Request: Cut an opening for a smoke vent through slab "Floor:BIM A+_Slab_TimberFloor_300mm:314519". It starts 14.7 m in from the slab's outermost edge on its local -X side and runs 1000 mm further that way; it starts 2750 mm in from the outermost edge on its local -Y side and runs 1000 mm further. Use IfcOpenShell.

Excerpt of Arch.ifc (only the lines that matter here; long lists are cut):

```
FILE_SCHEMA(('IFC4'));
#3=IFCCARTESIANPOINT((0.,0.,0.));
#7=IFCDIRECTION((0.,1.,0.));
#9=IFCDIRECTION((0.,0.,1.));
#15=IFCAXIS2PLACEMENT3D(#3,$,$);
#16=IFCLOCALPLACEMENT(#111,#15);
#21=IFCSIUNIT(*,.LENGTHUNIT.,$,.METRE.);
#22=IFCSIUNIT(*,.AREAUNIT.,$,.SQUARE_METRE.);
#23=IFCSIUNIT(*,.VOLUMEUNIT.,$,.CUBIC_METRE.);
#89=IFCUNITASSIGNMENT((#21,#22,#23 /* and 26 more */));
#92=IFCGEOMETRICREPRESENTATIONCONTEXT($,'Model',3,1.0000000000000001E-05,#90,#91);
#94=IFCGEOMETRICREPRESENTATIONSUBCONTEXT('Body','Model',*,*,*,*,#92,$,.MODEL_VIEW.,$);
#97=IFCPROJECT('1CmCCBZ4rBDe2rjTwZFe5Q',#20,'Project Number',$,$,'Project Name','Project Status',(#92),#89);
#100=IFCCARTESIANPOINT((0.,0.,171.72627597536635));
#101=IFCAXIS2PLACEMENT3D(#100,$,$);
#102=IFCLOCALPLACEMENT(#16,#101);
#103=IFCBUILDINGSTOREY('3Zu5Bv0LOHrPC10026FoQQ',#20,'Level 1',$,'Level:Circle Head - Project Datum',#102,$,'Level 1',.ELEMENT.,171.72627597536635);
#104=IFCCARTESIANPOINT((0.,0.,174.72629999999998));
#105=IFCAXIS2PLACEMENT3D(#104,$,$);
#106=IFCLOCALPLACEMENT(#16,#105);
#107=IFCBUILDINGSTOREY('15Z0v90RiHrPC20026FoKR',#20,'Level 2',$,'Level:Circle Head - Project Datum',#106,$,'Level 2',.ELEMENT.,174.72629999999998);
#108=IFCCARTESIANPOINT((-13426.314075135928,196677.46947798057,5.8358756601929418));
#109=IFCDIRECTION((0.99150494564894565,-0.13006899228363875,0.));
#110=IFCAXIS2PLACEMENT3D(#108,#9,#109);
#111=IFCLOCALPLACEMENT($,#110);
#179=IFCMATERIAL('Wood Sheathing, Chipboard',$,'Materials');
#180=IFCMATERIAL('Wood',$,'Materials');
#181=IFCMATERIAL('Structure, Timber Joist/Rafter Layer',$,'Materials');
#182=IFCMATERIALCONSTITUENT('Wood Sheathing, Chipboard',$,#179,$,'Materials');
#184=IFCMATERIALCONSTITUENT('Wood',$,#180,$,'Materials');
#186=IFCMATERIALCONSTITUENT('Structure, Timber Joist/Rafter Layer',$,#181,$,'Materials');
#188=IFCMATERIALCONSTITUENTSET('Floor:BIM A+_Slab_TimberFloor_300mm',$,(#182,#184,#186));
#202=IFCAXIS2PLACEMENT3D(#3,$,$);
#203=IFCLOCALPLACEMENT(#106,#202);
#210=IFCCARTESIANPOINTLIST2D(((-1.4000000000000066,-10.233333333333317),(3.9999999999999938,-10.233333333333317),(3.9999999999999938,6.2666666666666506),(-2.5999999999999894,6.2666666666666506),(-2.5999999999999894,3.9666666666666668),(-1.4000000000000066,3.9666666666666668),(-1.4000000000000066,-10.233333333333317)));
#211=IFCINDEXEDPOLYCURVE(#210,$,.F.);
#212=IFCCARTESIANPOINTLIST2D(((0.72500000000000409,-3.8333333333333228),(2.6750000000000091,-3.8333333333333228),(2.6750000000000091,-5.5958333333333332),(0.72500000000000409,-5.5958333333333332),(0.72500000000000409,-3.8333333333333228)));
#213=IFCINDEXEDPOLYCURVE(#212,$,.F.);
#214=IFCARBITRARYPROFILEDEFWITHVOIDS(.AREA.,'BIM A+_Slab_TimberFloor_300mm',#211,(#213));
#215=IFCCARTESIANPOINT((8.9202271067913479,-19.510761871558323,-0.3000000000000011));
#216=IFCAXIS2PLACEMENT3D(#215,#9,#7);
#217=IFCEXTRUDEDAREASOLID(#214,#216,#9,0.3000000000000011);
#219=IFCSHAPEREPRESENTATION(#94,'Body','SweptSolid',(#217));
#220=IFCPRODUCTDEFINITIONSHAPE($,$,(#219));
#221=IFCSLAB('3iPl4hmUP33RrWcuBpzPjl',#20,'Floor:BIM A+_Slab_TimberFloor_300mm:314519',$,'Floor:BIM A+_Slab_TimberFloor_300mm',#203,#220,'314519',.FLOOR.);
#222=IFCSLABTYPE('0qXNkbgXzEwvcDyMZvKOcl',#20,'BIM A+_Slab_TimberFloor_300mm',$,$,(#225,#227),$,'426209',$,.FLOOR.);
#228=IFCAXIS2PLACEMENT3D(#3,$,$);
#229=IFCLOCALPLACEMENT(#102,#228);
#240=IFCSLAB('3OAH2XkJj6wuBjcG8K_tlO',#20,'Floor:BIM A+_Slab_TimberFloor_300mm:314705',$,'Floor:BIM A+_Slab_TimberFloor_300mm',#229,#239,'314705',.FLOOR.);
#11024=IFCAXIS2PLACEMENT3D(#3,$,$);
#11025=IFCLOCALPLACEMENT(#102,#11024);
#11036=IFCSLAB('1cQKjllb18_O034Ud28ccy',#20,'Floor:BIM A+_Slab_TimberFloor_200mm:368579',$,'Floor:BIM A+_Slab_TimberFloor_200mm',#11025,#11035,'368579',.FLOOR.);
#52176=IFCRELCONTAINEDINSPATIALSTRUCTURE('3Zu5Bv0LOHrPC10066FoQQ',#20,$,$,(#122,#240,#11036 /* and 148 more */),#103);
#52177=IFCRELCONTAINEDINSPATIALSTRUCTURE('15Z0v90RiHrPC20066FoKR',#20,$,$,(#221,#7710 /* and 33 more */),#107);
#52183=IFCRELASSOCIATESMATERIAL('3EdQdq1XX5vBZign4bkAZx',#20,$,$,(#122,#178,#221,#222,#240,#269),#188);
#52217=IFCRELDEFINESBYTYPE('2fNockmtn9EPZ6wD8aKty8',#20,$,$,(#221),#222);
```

```python
import numpy as np
import ifcopenshell
import ifcopenshell.api.feature
import ifcopenshell.api.geometry
import ifcopenshell.api.root
import ifcopenshell.geom
import ifcopenshell.util.placement
import ifcopenshell.util.representation
import ifcopenshell.util.shape
import ifcopenshell.util.unit

model = ifcopenshell.open("Arch.ifc")
unit_scale = ifcopenshell.util.unit.calculate_unit_scale(model)
settings = ifcopenshell.geom.settings()


def volume(element):
    """Net volume in cubic metres, openings subtracted."""
    shape = ifcopenshell.geom.create_shape(settings, element)
    return ifcopenshell.util.shape.get_volume(shape.geometry)


slab = model.by_guid("3iPl4hmUP33RrWcuBpzPjl")
before = volume(slab)

# Extent in the slab's own axes, in metres. The edges named are its -X and -Y sides.
slab_shape = ifcopenshell.geom.create_shape(settings, slab)
vertices = ifcopenshell.util.shape.get_vertices(slab_shape.geometry)
x_min, y_min, bottom = vertices.min(axis=0)
top = vertices[:, 2].max()

opening = ifcopenshell.api.root.create_entity(model, ifc_class="IfcOpeningElement", name="Smoke vent opening", predefined_type="OPENING")
context = ifcopenshell.util.representation.get_context(model, "Model", "Body", "MODEL_VIEW")
width, depth = 1, 1
outline = [(0.0, 0.0), (width, 0.0), (width, depth), (0.0, depth), (0.0, 0.0)]
# Overshoot both faces by 50 mm so the cut is clean.
shape = ifcopenshell.api.geometry.add_slab_representation(
    model, context=context, depth=top - bottom + 0.1, polyline=outline
)
ifcopenshell.api.geometry.assign_representation(model, product=opening, representation=shape)

matrix = ifcopenshell.util.placement.get_local_placement(slab.ObjectPlacement)
matrix[:, 3] = matrix @ np.append(np.array([x_min + 14.7, y_min + 2.75, bottom - 0.05]) / unit_scale, 1.0)
ifcopenshell.api.geometry.edit_object_placement(model, product=opening, matrix=matrix, is_si=False)
ifcopenshell.api.feature.add_feature(model, feature=opening, element=slab)

after = volume(slab)

print(f"slab volume {before:.3f} -> {after:.3f} m3")

model.write("Arch_edited.ifc")
```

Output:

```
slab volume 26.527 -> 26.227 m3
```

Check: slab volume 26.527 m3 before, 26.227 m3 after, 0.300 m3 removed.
